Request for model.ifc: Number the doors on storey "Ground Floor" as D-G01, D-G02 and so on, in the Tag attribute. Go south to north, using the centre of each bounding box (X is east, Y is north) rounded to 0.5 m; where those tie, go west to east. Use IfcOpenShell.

First a look at what the model holds.

```python
import ifcopenshell
import ifcopenshell.util.element
import ifcopenshell.util.placement

model = ifcopenshell.open("model.ifc")
print(model.schema)
storey = next(s for s in model.by_type("IfcBuildingStorey") if s.Name == "Ground Floor")
doors = [e for e in ifcopenshell.util.element.get_decomposition(storey) if e.is_a("IfcDoor")]
for e in sorted(doors, key=lambda e: e.id()):
    origin = ifcopenshell.util.placement.get_local_placement(e.ObjectPlacement)[:3, 3]
    print(e.id(), e.Tag, e.Name, origin.round(2) + 0.0, sep=" | ")
```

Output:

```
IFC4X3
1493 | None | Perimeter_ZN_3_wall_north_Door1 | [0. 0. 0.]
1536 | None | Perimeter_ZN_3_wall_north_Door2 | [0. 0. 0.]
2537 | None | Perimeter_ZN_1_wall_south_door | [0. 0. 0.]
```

```python
import ifcopenshell
import ifcopenshell.geom
import ifcopenshell.util.element
import ifcopenshell.util.shape

model = ifcopenshell.open("model.ifc")
settings = ifcopenshell.geom.settings()
settings.set("use-world-coords", True)


def centre(element):
    shape = ifcopenshell.geom.create_shape(settings, element)
    return ifcopenshell.util.shape.get_bbox_centroid(shape.geometry)


storey = next(s for s in model.by_type("IfcBuildingStorey") if s.Name == "Ground Floor")
doors = [e for e in ifcopenshell.util.element.get_decomposition(storey) if e.is_a("IfcDoor")]

# Insertion points can sit at a corner or the storey origin, so sort by the geometry (in metres).
centres = {e: centre(e) for e in doors}
doors.sort(key=lambda e: (round(centres[e][1] / 0.5), centres[e][0]))

for i, e in enumerate(doors, start=1):
    number = f"D-G{i:02d}"
    e.Tag = number
    print(e.id(), number)

model.write("model_v2.ifc")
```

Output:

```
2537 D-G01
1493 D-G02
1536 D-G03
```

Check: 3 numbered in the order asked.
